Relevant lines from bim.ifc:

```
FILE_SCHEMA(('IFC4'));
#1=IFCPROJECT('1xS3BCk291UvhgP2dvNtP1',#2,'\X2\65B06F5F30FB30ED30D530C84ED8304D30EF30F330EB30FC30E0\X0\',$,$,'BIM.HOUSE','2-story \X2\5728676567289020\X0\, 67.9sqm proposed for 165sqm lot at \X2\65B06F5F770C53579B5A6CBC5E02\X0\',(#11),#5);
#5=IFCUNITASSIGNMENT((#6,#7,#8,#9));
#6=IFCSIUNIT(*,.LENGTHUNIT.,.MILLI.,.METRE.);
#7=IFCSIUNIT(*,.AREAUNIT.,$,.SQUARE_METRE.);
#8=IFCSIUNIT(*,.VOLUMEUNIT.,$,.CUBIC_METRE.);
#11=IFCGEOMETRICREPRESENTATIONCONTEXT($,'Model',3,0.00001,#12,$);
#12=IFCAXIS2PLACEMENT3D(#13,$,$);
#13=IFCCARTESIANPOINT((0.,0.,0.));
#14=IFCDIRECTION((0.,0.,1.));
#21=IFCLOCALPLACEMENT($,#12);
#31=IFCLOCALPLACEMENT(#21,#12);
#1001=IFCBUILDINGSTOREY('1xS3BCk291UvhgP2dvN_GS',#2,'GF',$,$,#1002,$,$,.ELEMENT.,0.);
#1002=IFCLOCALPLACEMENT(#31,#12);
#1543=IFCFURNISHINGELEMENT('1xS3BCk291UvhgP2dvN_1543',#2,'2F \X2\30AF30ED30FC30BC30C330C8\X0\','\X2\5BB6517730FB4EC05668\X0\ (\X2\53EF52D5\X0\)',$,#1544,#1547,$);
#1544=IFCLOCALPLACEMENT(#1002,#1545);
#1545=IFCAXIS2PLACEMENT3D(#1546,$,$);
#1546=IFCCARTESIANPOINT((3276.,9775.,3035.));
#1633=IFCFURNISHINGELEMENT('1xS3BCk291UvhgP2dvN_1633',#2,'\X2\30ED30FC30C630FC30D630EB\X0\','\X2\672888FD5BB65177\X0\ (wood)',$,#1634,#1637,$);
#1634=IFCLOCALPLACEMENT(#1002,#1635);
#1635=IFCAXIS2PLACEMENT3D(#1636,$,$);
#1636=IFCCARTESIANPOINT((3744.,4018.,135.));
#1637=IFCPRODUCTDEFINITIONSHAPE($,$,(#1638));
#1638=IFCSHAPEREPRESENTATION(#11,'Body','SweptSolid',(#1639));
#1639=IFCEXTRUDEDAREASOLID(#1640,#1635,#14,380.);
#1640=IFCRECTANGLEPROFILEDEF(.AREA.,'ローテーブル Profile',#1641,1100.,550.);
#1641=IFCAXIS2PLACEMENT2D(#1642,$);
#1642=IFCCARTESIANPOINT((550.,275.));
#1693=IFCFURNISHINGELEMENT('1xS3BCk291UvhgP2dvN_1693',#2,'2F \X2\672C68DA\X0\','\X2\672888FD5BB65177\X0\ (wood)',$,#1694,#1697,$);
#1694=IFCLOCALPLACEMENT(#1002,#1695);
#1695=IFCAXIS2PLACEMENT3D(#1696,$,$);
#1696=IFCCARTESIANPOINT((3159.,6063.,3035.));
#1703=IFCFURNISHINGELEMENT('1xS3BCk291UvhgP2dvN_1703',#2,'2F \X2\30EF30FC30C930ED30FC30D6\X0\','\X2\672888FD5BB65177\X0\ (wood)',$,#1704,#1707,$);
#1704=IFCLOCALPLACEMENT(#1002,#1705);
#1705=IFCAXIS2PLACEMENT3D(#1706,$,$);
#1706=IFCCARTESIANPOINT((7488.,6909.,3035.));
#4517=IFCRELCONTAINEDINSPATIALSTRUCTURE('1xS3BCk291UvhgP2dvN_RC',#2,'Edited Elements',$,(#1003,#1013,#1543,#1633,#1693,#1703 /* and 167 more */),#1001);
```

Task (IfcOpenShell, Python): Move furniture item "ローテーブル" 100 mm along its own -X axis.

```python
import ifcopenshell
import ifcopenshell.api.geometry
import ifcopenshell.util.placement

model = ifcopenshell.open("bim.ifc")

item = model.by_guid("1xS3BCk291UvhgP2dvN_1633")
matrix = ifcopenshell.util.placement.get_local_placement(item.ObjectPlacement)
matrix[:3, 3] -= matrix[:3, 0] * 100.0
ifcopenshell.api.geometry.edit_object_placement(model, product=item, matrix=matrix, is_si=False)

print(ifcopenshell.util.placement.get_local_placement(item.ObjectPlacement).round(3) + 0.0)

model.write("bim_v2.ifc")
```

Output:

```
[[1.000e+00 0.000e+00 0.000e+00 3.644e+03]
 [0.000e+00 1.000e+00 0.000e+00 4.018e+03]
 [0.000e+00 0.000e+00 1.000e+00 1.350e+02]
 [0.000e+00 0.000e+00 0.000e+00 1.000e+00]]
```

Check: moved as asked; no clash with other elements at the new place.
